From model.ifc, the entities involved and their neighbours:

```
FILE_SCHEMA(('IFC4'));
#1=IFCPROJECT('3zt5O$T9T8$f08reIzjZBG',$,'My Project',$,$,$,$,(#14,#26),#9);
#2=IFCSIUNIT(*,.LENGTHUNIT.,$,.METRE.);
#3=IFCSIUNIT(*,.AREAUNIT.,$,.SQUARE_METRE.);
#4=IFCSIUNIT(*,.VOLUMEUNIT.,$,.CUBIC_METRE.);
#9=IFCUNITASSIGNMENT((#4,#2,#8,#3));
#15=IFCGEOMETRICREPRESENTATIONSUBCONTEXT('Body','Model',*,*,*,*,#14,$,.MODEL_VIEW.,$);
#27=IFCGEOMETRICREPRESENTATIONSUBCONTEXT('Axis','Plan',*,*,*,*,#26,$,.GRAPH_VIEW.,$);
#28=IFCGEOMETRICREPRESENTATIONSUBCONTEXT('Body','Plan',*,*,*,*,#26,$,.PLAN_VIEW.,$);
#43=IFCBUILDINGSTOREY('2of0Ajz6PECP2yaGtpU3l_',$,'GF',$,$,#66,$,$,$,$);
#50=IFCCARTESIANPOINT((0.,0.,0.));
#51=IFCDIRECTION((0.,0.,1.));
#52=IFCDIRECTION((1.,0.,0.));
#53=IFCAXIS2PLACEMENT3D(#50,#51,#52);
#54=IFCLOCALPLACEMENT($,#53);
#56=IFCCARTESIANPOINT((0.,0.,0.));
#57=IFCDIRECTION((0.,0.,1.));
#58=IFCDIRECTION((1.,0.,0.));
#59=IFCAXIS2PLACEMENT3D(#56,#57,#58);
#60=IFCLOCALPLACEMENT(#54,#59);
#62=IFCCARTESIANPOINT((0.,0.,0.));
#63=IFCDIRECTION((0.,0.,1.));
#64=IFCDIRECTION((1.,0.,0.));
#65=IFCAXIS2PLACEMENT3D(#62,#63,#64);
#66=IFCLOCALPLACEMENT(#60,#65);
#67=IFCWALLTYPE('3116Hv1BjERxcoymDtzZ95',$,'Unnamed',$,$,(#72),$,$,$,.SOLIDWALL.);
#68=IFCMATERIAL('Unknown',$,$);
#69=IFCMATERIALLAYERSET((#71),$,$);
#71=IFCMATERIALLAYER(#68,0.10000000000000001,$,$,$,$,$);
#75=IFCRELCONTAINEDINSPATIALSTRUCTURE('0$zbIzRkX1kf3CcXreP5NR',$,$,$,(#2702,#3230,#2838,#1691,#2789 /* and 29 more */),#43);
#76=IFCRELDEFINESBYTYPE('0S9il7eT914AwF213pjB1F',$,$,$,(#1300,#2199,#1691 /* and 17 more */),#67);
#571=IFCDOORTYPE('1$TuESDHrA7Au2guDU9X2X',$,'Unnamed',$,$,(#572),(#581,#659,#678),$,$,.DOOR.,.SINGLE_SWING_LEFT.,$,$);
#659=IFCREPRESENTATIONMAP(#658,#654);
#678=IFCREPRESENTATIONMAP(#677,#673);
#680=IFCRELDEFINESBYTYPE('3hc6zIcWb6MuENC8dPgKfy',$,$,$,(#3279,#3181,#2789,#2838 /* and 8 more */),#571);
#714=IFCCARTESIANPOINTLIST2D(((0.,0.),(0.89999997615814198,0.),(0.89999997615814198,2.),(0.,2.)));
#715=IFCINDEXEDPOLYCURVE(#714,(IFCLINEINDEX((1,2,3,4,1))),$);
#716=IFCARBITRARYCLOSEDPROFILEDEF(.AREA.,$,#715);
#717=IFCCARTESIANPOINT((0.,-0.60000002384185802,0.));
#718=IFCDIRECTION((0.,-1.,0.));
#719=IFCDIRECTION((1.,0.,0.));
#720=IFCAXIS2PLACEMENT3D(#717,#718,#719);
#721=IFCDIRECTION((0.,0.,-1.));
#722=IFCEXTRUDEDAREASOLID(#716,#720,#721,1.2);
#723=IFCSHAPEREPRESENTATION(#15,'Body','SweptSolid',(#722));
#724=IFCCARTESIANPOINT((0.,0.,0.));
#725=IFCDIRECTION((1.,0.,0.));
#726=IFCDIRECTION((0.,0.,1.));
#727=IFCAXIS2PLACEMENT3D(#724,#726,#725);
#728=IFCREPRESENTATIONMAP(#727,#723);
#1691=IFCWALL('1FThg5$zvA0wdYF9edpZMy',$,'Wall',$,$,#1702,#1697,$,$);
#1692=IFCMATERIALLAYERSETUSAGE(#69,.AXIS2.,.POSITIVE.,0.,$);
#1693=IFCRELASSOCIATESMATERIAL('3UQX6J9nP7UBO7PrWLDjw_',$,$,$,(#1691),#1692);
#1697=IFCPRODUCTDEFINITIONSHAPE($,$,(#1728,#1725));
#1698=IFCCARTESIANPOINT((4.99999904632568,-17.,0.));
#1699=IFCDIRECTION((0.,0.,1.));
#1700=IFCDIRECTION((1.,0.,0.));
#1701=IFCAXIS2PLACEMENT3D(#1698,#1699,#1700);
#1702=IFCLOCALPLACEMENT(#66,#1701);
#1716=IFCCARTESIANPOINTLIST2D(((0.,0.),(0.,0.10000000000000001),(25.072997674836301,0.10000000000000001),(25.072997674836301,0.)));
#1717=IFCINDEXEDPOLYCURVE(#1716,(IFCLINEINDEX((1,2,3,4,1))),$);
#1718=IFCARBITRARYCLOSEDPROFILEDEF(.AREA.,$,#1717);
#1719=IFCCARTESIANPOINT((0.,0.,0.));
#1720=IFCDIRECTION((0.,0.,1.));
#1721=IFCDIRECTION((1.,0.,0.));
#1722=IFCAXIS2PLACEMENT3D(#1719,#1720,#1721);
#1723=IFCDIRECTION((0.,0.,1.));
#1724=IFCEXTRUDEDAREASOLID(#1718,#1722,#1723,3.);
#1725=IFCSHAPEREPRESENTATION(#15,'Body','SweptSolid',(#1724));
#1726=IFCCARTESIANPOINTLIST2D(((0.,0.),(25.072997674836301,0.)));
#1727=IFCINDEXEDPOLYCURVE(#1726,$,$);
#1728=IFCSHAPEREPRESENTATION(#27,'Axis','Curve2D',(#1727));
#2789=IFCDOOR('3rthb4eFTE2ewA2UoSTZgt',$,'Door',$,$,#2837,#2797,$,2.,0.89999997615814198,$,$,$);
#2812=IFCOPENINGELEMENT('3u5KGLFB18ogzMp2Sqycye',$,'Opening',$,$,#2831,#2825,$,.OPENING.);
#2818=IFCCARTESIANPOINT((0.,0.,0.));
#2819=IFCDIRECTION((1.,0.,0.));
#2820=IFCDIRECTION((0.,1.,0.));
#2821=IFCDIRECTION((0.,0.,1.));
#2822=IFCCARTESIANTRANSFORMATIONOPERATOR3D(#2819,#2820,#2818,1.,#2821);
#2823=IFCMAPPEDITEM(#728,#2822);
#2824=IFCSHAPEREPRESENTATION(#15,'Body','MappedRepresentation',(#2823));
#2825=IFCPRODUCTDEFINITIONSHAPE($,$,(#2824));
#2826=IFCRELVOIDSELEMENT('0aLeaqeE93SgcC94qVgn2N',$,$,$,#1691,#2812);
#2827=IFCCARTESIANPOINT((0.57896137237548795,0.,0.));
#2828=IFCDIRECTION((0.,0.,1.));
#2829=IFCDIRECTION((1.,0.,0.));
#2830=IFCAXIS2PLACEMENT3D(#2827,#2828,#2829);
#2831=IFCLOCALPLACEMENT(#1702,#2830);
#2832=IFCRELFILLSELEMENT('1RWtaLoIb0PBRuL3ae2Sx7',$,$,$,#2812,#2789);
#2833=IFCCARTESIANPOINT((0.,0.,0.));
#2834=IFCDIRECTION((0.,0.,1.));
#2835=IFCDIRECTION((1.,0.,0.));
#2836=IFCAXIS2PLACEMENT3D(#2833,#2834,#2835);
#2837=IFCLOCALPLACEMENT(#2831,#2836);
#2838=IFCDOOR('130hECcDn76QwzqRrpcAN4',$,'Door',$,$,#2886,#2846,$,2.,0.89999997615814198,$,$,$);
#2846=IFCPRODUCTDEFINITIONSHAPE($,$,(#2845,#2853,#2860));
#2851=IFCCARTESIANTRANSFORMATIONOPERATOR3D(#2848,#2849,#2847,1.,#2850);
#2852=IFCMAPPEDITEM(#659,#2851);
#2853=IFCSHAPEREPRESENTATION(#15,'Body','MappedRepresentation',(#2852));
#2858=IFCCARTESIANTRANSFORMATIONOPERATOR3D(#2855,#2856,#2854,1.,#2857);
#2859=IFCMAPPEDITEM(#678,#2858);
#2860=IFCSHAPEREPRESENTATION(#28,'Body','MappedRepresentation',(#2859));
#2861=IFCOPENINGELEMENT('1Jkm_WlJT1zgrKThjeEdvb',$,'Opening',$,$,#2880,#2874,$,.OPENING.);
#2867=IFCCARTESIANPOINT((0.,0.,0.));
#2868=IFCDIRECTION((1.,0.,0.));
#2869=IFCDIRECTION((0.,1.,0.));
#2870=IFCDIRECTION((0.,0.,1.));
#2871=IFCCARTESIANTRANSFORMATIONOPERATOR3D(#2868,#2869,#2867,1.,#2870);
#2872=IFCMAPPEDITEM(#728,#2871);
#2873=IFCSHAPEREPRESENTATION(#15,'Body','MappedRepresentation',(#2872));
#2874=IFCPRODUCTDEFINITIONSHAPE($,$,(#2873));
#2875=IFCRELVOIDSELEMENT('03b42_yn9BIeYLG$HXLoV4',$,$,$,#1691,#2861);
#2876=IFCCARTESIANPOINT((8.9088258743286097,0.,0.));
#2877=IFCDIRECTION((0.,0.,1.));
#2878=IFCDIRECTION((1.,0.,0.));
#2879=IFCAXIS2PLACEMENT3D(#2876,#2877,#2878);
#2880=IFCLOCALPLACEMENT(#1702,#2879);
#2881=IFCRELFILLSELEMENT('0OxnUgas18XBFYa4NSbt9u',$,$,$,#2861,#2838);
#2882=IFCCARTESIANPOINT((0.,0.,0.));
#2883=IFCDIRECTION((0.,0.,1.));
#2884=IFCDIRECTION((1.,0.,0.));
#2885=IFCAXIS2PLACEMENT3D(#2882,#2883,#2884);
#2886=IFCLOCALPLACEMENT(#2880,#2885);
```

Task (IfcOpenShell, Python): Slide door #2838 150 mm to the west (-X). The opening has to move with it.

```python
import ifcopenshell
import ifcopenshell.api.geometry
import ifcopenshell.util.placement
import ifcopenshell.util.unit

model = ifcopenshell.open("model.ifc")
unit_scale = ifcopenshell.util.unit.calculate_unit_scale(model)

door = model.by_guid("130hECcDn76QwzqRrpcAN4")
opening = door.FillsVoids[0].RelatingOpeningElement
wall = opening.VoidsElements[0].RelatingBuildingElement

wall_matrix = ifcopenshell.util.placement.get_local_placement(wall.ObjectPlacement)
shift = wall_matrix[:3, 0] * -0.15 / unit_scale
before = ifcopenshell.util.placement.get_local_placement(door.ObjectPlacement)[:3, 3].copy()

# The door is placed relative to its opening, so it follows when the opening moves.
matrix = ifcopenshell.util.placement.get_local_placement(opening.ObjectPlacement)
matrix[:3, 3] += shift
ifcopenshell.api.geometry.edit_object_placement(
    model, product=opening, matrix=matrix, is_si=False, should_transform_children=True
)

after = ifcopenshell.util.placement.get_local_placement(door.ObjectPlacement)[:3, 3]
print("door moved by", (after - before).round(3) + 0.0)

model.write("model_rev.ifc")
```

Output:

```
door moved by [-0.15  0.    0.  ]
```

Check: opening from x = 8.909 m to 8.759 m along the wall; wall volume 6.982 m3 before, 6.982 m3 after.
